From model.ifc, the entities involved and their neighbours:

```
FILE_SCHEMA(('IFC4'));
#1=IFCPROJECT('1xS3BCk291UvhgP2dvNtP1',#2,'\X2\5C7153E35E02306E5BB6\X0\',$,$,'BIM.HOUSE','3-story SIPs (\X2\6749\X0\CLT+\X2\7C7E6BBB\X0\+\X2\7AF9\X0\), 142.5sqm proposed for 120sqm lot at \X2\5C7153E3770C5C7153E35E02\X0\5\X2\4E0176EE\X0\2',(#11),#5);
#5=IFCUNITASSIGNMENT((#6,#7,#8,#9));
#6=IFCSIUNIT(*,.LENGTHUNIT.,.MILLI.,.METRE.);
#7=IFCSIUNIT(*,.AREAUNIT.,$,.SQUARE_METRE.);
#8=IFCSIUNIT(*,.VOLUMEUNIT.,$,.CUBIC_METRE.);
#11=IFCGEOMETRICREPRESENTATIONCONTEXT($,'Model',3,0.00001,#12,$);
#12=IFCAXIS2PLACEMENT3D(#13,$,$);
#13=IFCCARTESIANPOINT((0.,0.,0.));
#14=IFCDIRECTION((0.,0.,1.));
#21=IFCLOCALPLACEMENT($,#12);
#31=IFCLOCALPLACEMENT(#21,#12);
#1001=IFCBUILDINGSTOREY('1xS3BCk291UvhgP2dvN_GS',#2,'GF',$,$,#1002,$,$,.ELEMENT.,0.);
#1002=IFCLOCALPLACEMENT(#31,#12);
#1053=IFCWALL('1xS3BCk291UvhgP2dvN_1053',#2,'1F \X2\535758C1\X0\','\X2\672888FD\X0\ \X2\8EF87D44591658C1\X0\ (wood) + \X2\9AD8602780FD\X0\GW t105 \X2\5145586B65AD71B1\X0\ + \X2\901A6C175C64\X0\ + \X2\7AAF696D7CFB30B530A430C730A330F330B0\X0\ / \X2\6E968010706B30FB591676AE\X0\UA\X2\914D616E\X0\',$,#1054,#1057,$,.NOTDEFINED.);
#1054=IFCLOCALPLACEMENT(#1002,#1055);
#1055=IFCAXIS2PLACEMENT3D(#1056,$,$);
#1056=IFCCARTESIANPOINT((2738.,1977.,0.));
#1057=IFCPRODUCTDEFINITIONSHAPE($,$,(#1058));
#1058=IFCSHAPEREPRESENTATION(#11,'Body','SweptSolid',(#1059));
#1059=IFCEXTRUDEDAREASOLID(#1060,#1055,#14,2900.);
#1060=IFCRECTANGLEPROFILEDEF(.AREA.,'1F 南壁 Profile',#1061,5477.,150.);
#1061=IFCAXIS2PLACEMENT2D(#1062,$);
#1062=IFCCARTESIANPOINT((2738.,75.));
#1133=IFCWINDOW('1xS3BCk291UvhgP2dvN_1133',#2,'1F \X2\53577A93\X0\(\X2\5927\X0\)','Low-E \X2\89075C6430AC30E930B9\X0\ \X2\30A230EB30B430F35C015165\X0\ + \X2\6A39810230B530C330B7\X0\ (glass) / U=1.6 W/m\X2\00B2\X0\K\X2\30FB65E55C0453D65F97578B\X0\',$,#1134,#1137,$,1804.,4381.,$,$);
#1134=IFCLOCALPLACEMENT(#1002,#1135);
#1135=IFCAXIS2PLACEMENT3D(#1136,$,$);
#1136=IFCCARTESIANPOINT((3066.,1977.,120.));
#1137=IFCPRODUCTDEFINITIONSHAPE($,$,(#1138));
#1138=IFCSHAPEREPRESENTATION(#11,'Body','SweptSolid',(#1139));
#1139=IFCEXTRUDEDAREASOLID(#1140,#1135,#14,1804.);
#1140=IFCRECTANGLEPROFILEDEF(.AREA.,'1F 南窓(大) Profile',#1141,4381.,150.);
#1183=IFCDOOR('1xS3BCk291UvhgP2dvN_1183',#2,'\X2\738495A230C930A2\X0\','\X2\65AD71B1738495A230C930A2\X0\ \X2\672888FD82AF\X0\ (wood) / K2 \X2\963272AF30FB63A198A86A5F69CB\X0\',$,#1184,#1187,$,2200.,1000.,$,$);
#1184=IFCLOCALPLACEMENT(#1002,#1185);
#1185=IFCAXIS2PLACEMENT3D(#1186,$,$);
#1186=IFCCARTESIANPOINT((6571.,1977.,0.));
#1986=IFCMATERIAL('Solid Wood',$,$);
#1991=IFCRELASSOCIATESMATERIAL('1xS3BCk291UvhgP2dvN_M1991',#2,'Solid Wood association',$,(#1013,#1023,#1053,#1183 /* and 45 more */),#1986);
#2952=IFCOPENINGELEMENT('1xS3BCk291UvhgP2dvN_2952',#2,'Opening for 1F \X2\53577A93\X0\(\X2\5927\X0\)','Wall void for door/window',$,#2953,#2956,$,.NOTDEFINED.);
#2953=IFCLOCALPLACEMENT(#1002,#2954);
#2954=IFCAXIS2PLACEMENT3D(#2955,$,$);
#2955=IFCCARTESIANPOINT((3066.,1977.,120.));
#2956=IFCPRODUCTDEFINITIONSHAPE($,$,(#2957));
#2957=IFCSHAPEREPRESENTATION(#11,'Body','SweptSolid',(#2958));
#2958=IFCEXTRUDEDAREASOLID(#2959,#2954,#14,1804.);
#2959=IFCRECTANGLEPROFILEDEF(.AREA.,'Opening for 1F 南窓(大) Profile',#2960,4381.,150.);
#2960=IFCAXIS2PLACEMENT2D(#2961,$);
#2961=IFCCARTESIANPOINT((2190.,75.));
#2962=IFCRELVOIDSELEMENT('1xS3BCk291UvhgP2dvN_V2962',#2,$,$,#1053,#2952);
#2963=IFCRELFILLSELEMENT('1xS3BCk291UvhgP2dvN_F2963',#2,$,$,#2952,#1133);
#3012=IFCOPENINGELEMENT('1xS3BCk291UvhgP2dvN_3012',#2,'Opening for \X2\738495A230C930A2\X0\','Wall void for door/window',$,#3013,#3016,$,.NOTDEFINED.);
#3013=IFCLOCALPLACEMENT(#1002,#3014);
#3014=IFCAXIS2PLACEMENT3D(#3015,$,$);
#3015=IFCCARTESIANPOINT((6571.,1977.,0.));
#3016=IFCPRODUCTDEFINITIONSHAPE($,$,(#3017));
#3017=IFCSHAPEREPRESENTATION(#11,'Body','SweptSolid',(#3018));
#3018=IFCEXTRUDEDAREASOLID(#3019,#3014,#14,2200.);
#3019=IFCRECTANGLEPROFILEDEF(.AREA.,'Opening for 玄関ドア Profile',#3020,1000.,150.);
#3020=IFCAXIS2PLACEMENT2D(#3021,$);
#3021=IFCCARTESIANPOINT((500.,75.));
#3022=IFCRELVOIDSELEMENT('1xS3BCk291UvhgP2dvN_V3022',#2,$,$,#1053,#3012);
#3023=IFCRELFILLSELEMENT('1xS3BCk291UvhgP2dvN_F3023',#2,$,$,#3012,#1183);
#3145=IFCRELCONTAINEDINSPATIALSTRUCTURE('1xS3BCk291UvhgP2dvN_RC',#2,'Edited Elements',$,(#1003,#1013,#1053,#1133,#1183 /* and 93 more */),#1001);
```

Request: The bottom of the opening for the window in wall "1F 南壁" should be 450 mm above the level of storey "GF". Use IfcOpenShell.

```python
import numpy as np
import ifcopenshell
import ifcopenshell.api.geometry
import ifcopenshell.geom
import ifcopenshell.util.element
import ifcopenshell.util.placement
import ifcopenshell.util.shape
import ifcopenshell.util.unit

model = ifcopenshell.open("model.ifc")
unit_scale = ifcopenshell.util.unit.calculate_unit_scale(model)

window = model.by_id(1133)
opening = window.FillsVoids[0].RelatingOpeningElement
storey = ifcopenshell.util.element.get_container(window, ifc_class="IfcBuildingStorey")
level = ifcopenshell.util.placement.get_local_placement(storey.ObjectPlacement)[2, 3]

# The opening's origin need not be at the sill, so measure its lowest point.
shape = ifcopenshell.geom.create_shape(ifcopenshell.geom.settings(), opening)
bottom = ifcopenshell.util.shape.get_shape_bottom_elevation(shape, shape.geometry) / unit_scale
dz = level + 450.0 - bottom

shift = np.array([0.0, 0.0, dz])
# The window is not placed relative to its opening, so move both.
for product in (opening, window):
    matrix = ifcopenshell.util.placement.get_local_placement(product.ObjectPlacement)
    matrix[:3, 3] += shift
    ifcopenshell.api.geometry.edit_object_placement(model, product=product, matrix=matrix, is_si=False)

print(f"moved by {dz * unit_scale:+.3f} m")

model.write("model-out.ifc")
```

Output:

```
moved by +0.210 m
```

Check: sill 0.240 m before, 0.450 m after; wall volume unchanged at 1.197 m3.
